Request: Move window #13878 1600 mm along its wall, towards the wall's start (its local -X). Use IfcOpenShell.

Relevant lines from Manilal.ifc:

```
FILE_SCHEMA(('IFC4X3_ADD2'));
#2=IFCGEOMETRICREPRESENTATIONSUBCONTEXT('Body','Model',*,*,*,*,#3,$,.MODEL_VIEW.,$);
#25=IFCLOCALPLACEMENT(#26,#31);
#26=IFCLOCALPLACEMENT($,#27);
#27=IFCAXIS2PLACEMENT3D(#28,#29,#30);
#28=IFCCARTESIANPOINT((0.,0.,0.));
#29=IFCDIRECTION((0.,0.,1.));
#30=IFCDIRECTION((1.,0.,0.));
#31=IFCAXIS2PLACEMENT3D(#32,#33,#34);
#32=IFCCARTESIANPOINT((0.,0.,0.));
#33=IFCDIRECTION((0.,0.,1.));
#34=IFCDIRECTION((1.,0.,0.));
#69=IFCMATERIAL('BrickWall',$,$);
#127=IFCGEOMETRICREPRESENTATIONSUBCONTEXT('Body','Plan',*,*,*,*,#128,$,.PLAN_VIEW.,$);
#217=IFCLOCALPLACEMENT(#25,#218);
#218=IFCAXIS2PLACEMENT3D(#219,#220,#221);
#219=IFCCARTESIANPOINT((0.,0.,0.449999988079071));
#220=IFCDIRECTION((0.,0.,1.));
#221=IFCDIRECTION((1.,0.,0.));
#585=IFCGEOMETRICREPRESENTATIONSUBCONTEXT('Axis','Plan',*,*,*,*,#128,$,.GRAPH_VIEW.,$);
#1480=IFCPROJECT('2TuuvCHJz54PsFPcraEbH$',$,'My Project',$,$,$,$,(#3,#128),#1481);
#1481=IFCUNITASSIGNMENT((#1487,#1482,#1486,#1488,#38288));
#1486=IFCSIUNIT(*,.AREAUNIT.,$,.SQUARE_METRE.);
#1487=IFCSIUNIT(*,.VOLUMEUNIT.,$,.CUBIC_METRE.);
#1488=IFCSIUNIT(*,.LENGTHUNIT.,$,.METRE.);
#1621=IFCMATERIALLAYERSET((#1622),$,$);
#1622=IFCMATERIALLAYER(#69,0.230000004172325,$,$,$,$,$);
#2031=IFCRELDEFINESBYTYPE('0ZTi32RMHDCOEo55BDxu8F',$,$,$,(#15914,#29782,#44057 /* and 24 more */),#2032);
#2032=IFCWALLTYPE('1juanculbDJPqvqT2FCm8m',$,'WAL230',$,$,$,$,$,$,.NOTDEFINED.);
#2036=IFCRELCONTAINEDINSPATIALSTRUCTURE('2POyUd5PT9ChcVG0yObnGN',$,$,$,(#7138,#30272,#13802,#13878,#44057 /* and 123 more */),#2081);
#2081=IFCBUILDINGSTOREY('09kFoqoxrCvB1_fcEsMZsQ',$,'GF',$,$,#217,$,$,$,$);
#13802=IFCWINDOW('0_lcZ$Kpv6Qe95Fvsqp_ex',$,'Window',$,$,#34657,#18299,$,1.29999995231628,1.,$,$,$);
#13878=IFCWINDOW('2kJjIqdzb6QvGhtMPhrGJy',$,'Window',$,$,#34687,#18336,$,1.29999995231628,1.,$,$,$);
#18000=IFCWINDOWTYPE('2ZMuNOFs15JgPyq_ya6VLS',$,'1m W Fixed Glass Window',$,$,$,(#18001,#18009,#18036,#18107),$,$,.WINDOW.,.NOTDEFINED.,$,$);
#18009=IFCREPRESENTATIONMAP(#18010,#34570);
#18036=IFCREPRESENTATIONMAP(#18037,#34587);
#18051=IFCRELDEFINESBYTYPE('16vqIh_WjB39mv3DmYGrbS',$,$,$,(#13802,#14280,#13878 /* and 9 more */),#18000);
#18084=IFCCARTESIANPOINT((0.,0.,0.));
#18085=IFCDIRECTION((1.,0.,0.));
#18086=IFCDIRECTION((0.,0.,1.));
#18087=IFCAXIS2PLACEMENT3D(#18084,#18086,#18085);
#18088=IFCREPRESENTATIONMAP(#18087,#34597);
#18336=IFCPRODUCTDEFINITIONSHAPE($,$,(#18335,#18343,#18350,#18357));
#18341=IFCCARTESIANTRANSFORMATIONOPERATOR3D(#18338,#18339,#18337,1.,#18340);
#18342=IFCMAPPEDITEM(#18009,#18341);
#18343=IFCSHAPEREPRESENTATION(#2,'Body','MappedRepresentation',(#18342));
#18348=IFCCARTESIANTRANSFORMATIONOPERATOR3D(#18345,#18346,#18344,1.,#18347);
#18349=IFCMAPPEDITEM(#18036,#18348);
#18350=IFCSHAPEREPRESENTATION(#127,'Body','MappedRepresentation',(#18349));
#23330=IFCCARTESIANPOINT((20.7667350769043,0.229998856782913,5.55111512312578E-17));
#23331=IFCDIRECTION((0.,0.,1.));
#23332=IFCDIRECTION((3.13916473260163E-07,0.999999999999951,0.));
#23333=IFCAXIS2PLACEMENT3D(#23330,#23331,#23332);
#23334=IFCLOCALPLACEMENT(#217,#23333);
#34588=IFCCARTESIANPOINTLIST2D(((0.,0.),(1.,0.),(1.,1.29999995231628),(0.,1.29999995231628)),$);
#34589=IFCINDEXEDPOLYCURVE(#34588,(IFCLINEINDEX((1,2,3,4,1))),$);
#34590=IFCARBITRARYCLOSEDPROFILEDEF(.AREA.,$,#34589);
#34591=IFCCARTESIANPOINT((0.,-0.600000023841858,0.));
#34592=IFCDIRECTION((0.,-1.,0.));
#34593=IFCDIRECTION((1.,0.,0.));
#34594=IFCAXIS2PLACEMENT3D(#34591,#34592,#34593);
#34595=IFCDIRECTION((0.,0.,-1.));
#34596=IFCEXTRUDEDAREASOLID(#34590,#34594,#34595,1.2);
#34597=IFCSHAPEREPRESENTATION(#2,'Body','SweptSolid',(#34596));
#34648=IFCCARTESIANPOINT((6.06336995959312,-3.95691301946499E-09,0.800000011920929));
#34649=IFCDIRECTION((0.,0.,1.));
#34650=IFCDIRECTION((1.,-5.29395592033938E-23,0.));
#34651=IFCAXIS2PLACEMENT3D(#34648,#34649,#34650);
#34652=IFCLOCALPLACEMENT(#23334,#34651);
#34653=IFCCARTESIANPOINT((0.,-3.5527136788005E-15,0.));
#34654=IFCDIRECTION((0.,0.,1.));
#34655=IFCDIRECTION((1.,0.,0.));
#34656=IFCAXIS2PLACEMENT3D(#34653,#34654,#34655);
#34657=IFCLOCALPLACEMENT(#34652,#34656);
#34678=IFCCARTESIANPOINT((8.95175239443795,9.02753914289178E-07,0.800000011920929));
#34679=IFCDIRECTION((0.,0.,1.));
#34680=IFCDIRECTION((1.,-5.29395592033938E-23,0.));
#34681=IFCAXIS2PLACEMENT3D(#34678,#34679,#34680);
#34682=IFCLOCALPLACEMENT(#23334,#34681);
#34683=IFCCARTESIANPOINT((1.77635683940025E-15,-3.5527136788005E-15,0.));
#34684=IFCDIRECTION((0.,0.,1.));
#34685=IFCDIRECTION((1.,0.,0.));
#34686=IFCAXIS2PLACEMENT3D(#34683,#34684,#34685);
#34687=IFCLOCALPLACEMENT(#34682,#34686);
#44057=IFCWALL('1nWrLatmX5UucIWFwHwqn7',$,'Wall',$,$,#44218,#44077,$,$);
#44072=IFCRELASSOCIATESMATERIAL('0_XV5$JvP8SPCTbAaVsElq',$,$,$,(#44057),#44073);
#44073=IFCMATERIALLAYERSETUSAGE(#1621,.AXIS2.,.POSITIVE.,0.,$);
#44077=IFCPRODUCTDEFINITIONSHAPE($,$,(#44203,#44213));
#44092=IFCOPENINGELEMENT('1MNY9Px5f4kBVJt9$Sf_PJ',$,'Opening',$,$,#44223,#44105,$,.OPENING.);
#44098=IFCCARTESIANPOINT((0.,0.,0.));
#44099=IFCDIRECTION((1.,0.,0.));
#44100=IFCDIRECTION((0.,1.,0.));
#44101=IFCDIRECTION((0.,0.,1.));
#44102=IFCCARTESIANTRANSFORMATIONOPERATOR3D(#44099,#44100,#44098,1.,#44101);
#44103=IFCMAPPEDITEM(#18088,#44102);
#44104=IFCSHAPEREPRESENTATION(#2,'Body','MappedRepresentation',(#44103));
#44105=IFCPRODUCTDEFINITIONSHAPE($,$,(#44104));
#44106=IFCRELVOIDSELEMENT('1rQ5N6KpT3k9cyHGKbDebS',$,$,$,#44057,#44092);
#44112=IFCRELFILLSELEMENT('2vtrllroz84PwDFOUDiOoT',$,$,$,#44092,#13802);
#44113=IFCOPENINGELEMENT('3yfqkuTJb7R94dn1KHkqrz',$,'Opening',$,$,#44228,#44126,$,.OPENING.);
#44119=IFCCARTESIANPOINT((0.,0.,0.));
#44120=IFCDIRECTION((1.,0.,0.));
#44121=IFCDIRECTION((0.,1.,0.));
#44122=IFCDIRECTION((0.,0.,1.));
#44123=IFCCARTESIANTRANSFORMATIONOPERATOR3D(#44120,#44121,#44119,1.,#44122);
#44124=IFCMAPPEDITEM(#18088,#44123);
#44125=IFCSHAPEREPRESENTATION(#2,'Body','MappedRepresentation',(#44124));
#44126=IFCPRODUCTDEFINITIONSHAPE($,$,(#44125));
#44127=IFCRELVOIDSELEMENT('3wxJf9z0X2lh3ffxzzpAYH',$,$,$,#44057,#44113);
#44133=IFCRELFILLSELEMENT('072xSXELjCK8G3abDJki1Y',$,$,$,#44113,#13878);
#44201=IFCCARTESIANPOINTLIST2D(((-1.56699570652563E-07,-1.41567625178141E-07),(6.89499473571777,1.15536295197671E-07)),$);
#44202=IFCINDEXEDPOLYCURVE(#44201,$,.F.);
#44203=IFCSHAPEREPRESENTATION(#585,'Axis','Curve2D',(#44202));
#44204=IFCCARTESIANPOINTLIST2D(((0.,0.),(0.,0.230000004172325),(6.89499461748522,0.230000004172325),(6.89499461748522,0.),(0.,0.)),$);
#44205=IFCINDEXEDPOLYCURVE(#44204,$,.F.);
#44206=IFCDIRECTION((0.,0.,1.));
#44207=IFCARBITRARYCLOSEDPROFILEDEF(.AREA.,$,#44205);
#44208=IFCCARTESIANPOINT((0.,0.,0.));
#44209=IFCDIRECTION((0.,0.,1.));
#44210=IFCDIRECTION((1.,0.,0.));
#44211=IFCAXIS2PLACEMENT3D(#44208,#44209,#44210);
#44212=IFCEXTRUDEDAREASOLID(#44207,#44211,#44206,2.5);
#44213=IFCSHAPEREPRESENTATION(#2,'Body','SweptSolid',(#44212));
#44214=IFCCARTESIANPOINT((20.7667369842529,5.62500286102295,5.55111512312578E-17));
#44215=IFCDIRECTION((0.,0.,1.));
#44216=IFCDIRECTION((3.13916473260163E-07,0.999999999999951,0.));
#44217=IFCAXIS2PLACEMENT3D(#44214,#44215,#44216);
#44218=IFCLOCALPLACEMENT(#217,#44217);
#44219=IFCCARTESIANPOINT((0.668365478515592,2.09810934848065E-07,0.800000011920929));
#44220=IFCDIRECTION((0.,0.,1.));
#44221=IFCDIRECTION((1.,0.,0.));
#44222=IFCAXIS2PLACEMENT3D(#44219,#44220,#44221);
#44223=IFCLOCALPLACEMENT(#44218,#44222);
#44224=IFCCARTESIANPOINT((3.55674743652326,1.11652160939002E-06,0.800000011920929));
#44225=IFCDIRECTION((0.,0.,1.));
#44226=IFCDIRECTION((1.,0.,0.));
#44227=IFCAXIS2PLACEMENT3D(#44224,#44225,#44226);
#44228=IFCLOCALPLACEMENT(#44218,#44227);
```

```python
import ifcopenshell
import ifcopenshell.api.geometry
import ifcopenshell.util.placement

model = ifcopenshell.open("Manilal.ifc")

window = model.by_guid("2kJjIqdzb6QvGhtMPhrGJy")
opening = window.FillsVoids[0].RelatingOpeningElement
wall = opening.VoidsElements[0].RelatingBuildingElement

wall_matrix = ifcopenshell.util.placement.get_local_placement(wall.ObjectPlacement)
shift = wall_matrix[:3, 0] * -1.6
before = ifcopenshell.util.placement.get_local_placement(window.ObjectPlacement)[:3, 3].copy()

# The window is not placed relative to its opening, so move both.
for product in (opening, window):
    matrix = ifcopenshell.util.placement.get_local_placement(product.ObjectPlacement)
    matrix[:3, 3] += shift
    ifcopenshell.api.geometry.edit_object_placement(model, product=product, matrix=matrix, is_si=False)

after = ifcopenshell.util.placement.get_local_placement(window.ObjectPlacement)[:3, 3]
print("window moved by", (after - before).round(3) + 0.0)

model.write("Manilal_rev.ifc")
```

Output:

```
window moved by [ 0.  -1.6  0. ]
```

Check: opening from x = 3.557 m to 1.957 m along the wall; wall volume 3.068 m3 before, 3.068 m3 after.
